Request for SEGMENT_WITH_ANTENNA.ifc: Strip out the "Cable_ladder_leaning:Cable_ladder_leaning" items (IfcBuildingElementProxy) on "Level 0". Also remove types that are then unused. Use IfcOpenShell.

First a look at what the model holds.

```python
import ifcopenshell
import ifcopenshell.util.element

model = ifcopenshell.open("SEGMENT_WITH_ANTENNA.ifc")
print(model.schema)
storey = next(s for s in model.by_type("IfcBuildingStorey") if s.Name == "Level 0")
proxies = [e for e in ifcopenshell.util.element.get_decomposition(storey) if e.is_a("IfcBuildingElementProxy")]
seen = {}
for e in proxies:
    element_type = ifcopenshell.util.element.get_type(e)
    name = element_type.Name if element_type not in (None, e) else None
    seen[name] = seen.get(name, 0) + 1
for name, count in sorted(seen.items(), key=str):
    print(count, "x", name)
```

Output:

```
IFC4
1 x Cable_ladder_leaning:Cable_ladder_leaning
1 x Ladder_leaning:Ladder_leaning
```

```python
import ifcopenshell
import ifcopenshell.api.root
import ifcopenshell.util.element

model = ifcopenshell.open("SEGMENT_WITH_ANTENNA.ifc")

storey = next(s for s in model.by_type("IfcBuildingStorey") if s.Name == "Level 0")
proxies = [e for e in ifcopenshell.util.element.get_decomposition(storey) if e.is_a("IfcBuildingElementProxy")]
targets = [e for e in proxies if (t := ifcopenshell.util.element.get_type(e)) not in (None, e) and t.Name == "Cable_ladder_leaning:Cable_ladder_leaning"]
types = {ifcopenshell.util.element.get_type(e) for e in targets} - {None, *targets}

for e in targets:
    ifcopenshell.api.root.remove_product(model, product=e)
print(len(targets), "removed")

unused = [t for t in types if not ifcopenshell.util.element.get_types(t)]
for t in unused:
    ifcopenshell.api.root.remove_product(model, product=t)
print(len(unused), "unused types removed")

model.write("SEGMENT_WITH_ANTENNA_updated.ifc")
```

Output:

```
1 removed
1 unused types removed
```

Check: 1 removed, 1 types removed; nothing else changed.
